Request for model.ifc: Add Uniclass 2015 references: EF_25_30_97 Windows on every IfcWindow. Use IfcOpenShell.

First a look at what the model holds.

```python
import ifcopenshell

model = ifcopenshell.open("model.ifc")
print(model.schema)
print("classifications:", [c.Name for c in model.by_type("IfcClassification")])
for ifc_class in ("IfcDoor", "IfcRoof", "IfcStair", "IfcWall", "IfcWindow"):
    print(ifc_class, len(model.by_type(ifc_class)))
```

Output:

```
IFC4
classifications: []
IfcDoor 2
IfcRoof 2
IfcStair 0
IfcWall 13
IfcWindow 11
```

```python
import ifcopenshell
import ifcopenshell.api.classification

model = ifcopenshell.open("model.ifc")

system = ifcopenshell.api.classification.add_classification(model, classification="Uniclass 2015")

codes = {
    "IfcWindow": ("EF_25_30_97", "Windows"),
}
for ifc_class, (code, name) in codes.items():
    products = model.by_type(ifc_class)
    ifcopenshell.api.classification.add_reference(
        model, products=products, classification=system, identification=code, name=name
    )
    print(code, len(products))

model.write("model_v2.ifc")
```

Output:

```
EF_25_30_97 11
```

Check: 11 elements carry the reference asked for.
